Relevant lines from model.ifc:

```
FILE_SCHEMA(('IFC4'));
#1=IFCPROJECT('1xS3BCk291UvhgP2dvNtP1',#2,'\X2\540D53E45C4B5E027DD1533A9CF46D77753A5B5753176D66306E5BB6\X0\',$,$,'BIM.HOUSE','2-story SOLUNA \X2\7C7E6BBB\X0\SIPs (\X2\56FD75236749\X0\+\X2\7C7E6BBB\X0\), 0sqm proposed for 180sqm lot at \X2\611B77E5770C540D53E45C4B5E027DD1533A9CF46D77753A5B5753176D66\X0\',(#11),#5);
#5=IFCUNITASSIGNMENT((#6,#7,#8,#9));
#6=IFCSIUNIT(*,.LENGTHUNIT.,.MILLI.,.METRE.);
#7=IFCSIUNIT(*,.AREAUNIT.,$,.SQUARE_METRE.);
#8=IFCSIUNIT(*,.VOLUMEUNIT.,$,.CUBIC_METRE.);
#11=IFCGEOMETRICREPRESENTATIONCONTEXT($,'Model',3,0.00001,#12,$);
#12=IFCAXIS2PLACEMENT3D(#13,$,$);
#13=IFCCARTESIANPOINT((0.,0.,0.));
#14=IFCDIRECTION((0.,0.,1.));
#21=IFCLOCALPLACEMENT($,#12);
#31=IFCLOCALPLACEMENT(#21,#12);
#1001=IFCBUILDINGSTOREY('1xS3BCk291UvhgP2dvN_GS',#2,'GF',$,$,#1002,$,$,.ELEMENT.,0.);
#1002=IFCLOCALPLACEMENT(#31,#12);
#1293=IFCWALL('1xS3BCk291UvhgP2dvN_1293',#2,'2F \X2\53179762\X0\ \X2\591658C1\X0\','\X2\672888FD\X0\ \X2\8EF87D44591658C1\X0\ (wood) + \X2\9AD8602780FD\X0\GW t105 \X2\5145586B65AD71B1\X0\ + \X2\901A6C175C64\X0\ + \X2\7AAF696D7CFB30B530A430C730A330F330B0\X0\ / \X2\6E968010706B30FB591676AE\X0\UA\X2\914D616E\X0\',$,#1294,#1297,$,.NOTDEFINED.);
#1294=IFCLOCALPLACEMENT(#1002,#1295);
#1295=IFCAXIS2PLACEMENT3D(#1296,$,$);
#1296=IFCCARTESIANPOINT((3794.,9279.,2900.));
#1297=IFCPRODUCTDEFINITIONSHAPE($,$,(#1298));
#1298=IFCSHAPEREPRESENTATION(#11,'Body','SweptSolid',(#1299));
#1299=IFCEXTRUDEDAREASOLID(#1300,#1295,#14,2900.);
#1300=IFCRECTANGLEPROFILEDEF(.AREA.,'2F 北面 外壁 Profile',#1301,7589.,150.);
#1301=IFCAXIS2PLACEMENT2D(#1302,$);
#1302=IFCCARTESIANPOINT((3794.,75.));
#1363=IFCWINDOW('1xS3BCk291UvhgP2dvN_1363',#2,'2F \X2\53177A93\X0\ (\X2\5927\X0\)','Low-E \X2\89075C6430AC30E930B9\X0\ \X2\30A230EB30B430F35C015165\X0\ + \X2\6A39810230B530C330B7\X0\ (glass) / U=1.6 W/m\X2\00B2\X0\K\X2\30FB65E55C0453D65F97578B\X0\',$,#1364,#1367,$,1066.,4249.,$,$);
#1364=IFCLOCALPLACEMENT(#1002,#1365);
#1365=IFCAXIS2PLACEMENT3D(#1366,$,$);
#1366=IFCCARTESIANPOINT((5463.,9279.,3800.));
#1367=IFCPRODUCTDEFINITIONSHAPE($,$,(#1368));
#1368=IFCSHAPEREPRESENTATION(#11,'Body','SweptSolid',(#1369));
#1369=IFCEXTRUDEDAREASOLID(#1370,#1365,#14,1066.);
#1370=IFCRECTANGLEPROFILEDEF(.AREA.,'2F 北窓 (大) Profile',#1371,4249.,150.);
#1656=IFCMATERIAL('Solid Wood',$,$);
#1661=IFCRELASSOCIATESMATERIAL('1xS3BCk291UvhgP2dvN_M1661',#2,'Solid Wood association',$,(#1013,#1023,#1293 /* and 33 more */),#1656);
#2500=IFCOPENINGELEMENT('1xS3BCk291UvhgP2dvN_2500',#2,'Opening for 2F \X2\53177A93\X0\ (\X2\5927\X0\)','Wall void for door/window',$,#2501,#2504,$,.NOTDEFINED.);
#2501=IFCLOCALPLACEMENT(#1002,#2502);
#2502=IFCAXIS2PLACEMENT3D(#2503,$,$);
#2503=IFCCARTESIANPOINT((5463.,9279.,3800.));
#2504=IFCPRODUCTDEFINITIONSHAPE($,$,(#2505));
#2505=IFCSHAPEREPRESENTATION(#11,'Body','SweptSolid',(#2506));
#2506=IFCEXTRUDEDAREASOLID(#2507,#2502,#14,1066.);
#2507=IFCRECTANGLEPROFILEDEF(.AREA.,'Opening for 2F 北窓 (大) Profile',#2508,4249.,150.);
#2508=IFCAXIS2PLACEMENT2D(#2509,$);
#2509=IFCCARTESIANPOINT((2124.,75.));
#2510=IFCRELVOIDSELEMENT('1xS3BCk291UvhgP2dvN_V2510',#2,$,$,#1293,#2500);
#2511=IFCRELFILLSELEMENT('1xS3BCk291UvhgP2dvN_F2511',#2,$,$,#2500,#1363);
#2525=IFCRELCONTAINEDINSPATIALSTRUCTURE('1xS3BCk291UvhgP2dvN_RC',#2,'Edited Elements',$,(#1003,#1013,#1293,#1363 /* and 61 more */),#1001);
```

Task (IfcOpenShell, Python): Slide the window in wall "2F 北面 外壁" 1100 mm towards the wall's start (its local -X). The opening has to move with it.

```python
import ifcopenshell
import ifcopenshell.api.geometry
import ifcopenshell.util.placement
import ifcopenshell.util.unit

model = ifcopenshell.open("model.ifc")
unit_scale = ifcopenshell.util.unit.calculate_unit_scale(model)

window = model.by_guid("1xS3BCk291UvhgP2dvN_1363")
opening = window.FillsVoids[0].RelatingOpeningElement
wall = opening.VoidsElements[0].RelatingBuildingElement

wall_matrix = ifcopenshell.util.placement.get_local_placement(wall.ObjectPlacement)
shift = wall_matrix[:3, 0] * -1.1 / unit_scale
before = ifcopenshell.util.placement.get_local_placement(window.ObjectPlacement)[:3, 3].copy()

# The window is not placed relative to its opening, so move both.
for product in (opening, window):
    matrix = ifcopenshell.util.placement.get_local_placement(product.ObjectPlacement)
    matrix[:3, 3] += shift
    ifcopenshell.api.geometry.edit_object_placement(model, product=product, matrix=matrix, is_si=False)

after = ifcopenshell.util.placement.get_local_placement(window.ObjectPlacement)[:3, 3]
print("window moved by", (after - before).round(3) + 0.0)

model.write("model-out.ifc")
```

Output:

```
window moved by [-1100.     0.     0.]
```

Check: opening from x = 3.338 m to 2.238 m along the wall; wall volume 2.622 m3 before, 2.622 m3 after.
